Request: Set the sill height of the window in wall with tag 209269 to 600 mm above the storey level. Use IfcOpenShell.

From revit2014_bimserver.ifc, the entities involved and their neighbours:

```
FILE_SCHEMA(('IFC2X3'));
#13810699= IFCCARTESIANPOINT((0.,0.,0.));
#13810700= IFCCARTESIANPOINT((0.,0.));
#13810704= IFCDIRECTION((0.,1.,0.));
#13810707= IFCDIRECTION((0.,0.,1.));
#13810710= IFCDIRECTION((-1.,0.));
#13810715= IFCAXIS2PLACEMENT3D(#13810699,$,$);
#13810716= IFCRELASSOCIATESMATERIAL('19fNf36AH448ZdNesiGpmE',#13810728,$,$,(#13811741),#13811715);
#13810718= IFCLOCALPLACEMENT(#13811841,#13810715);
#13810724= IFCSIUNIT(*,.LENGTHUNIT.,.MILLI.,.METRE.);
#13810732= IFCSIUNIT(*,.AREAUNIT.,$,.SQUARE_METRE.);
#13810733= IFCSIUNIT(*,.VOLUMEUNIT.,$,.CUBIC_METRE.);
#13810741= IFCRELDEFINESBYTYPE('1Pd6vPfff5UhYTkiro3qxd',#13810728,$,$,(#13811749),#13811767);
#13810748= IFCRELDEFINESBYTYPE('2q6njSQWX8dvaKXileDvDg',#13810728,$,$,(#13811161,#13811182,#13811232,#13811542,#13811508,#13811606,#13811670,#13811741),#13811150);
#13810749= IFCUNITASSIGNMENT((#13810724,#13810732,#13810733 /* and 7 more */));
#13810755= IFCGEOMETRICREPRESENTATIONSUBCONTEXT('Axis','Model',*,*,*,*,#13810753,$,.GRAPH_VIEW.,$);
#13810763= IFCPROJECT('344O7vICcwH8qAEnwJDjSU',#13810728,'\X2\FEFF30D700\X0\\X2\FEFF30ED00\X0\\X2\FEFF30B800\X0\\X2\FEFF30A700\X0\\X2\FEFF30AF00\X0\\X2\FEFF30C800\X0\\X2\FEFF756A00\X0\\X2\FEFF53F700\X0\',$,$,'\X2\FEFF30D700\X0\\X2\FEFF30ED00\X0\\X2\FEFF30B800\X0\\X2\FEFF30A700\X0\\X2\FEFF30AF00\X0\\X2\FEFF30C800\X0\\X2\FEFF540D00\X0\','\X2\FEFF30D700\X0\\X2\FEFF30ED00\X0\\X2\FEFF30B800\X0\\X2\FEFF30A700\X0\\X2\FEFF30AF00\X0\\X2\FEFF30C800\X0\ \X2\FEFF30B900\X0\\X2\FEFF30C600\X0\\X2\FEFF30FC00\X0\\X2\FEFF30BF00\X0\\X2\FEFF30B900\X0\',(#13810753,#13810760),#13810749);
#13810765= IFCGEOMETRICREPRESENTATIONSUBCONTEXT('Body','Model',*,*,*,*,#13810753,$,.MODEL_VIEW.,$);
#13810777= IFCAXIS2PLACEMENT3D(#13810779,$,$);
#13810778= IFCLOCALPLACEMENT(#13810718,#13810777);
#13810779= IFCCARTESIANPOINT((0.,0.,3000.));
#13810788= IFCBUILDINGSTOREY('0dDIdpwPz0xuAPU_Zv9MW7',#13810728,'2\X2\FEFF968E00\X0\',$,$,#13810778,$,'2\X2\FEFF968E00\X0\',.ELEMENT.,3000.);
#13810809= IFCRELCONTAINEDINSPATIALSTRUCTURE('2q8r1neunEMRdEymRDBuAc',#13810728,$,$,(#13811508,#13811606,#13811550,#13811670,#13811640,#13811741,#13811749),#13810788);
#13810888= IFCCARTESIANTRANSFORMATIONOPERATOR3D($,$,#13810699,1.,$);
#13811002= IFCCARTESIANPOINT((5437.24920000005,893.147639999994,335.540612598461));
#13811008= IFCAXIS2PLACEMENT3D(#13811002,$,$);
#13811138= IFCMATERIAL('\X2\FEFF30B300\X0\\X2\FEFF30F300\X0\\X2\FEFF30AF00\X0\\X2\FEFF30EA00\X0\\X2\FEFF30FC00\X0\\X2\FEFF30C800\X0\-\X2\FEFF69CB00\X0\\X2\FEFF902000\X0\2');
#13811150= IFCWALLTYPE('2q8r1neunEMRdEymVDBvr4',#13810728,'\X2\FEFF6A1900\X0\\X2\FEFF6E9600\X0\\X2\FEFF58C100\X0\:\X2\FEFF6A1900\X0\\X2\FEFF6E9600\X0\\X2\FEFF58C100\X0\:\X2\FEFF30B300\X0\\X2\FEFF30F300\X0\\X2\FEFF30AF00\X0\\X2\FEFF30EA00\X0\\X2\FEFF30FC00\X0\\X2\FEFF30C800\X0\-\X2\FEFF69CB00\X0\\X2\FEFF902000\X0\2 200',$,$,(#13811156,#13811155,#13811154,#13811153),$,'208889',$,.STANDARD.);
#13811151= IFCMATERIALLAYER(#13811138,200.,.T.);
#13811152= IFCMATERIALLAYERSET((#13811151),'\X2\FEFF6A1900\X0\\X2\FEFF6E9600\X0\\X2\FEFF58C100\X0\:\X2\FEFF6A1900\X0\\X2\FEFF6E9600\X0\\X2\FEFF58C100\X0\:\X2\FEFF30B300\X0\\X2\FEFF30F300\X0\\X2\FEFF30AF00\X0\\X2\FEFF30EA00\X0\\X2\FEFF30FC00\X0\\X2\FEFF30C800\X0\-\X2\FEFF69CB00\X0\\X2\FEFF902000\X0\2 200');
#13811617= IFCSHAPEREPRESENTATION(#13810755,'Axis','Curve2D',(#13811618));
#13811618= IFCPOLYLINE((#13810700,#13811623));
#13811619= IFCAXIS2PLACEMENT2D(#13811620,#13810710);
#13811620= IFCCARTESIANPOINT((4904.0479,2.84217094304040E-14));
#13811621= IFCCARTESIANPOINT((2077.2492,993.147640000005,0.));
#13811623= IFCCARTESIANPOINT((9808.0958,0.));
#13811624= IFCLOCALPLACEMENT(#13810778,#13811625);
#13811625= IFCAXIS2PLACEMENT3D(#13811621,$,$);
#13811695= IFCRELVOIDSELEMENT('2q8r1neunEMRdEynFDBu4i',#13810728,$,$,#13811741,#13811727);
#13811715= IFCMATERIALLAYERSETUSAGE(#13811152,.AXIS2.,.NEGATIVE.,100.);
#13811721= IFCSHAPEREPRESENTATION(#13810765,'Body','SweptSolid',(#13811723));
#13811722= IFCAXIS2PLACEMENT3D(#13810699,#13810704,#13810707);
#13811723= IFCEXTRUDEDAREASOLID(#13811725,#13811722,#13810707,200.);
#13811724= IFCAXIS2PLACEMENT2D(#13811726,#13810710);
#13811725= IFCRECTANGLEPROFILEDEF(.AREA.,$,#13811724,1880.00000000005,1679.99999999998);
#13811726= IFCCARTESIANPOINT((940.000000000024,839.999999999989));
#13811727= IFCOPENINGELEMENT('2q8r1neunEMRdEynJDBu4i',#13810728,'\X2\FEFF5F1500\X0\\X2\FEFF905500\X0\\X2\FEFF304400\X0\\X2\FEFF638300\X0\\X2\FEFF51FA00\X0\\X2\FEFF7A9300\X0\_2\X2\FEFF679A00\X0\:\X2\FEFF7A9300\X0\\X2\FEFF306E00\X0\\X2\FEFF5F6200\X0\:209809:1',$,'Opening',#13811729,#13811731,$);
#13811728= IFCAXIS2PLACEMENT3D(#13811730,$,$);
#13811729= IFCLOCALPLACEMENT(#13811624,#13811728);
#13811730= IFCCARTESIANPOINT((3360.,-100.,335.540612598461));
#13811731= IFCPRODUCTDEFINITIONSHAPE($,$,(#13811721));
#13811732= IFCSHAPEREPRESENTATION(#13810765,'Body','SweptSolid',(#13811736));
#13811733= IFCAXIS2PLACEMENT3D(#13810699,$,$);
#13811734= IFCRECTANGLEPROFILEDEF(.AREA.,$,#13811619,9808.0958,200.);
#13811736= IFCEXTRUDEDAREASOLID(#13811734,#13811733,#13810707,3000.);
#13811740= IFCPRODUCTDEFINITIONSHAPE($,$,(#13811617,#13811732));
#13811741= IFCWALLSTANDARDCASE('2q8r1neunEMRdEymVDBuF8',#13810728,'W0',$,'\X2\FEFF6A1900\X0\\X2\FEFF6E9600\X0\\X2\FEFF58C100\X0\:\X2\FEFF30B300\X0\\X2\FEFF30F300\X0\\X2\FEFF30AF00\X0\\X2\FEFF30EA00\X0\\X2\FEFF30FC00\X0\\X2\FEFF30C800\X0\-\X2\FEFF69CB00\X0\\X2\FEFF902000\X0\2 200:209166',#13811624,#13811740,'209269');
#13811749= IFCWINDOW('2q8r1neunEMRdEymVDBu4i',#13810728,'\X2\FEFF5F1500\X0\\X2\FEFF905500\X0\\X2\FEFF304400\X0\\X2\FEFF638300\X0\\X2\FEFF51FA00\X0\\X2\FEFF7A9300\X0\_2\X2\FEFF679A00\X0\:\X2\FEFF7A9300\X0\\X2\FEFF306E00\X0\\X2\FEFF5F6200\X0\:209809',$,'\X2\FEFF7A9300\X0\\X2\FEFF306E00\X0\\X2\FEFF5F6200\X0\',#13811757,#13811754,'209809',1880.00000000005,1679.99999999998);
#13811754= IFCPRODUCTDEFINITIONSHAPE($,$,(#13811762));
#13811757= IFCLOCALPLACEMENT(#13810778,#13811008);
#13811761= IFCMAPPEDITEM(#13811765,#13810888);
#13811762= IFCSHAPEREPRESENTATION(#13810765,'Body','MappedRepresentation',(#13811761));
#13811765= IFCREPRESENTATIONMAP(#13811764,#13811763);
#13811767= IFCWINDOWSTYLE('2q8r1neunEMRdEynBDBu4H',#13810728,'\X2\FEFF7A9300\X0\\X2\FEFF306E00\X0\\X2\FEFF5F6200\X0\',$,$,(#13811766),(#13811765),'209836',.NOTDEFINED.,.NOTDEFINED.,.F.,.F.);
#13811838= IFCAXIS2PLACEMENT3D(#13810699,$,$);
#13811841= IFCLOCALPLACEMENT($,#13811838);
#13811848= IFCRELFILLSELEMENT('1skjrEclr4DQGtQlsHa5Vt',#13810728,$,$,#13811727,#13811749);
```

```python
import numpy as np
import ifcopenshell
import ifcopenshell.api.geometry
import ifcopenshell.geom
import ifcopenshell.util.element
import ifcopenshell.util.placement
import ifcopenshell.util.shape
import ifcopenshell.util.unit

model = ifcopenshell.open("revit2014_bimserver.ifc")
unit_scale = ifcopenshell.util.unit.calculate_unit_scale(model)

window = model.by_guid("2q8r1neunEMRdEymVDBu4i")
opening = window.FillsVoids[0].RelatingOpeningElement
storey = ifcopenshell.util.element.get_container(window, ifc_class="IfcBuildingStorey")
level = ifcopenshell.util.placement.get_local_placement(storey.ObjectPlacement)[2, 3]

# The opening's origin need not be at the sill, so measure its lowest point.
shape = ifcopenshell.geom.create_shape(ifcopenshell.geom.settings(), opening)
bottom = ifcopenshell.util.shape.get_shape_bottom_elevation(shape, shape.geometry) / unit_scale
dz = level + 600.0 - bottom

shift = np.array([0.0, 0.0, dz])
# The window is not placed relative to its opening, so move both.
for product in (opening, window):
    matrix = ifcopenshell.util.placement.get_local_placement(product.ObjectPlacement)
    matrix[:3, 3] += shift
    ifcopenshell.api.geometry.edit_object_placement(model, product=product, matrix=matrix, is_si=False)

print(f"moved by {dz * unit_scale:+.3f} m")

model.write("revit2014_bimserver_edited.ifc")
```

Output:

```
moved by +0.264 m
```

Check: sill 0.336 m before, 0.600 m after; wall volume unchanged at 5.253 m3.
